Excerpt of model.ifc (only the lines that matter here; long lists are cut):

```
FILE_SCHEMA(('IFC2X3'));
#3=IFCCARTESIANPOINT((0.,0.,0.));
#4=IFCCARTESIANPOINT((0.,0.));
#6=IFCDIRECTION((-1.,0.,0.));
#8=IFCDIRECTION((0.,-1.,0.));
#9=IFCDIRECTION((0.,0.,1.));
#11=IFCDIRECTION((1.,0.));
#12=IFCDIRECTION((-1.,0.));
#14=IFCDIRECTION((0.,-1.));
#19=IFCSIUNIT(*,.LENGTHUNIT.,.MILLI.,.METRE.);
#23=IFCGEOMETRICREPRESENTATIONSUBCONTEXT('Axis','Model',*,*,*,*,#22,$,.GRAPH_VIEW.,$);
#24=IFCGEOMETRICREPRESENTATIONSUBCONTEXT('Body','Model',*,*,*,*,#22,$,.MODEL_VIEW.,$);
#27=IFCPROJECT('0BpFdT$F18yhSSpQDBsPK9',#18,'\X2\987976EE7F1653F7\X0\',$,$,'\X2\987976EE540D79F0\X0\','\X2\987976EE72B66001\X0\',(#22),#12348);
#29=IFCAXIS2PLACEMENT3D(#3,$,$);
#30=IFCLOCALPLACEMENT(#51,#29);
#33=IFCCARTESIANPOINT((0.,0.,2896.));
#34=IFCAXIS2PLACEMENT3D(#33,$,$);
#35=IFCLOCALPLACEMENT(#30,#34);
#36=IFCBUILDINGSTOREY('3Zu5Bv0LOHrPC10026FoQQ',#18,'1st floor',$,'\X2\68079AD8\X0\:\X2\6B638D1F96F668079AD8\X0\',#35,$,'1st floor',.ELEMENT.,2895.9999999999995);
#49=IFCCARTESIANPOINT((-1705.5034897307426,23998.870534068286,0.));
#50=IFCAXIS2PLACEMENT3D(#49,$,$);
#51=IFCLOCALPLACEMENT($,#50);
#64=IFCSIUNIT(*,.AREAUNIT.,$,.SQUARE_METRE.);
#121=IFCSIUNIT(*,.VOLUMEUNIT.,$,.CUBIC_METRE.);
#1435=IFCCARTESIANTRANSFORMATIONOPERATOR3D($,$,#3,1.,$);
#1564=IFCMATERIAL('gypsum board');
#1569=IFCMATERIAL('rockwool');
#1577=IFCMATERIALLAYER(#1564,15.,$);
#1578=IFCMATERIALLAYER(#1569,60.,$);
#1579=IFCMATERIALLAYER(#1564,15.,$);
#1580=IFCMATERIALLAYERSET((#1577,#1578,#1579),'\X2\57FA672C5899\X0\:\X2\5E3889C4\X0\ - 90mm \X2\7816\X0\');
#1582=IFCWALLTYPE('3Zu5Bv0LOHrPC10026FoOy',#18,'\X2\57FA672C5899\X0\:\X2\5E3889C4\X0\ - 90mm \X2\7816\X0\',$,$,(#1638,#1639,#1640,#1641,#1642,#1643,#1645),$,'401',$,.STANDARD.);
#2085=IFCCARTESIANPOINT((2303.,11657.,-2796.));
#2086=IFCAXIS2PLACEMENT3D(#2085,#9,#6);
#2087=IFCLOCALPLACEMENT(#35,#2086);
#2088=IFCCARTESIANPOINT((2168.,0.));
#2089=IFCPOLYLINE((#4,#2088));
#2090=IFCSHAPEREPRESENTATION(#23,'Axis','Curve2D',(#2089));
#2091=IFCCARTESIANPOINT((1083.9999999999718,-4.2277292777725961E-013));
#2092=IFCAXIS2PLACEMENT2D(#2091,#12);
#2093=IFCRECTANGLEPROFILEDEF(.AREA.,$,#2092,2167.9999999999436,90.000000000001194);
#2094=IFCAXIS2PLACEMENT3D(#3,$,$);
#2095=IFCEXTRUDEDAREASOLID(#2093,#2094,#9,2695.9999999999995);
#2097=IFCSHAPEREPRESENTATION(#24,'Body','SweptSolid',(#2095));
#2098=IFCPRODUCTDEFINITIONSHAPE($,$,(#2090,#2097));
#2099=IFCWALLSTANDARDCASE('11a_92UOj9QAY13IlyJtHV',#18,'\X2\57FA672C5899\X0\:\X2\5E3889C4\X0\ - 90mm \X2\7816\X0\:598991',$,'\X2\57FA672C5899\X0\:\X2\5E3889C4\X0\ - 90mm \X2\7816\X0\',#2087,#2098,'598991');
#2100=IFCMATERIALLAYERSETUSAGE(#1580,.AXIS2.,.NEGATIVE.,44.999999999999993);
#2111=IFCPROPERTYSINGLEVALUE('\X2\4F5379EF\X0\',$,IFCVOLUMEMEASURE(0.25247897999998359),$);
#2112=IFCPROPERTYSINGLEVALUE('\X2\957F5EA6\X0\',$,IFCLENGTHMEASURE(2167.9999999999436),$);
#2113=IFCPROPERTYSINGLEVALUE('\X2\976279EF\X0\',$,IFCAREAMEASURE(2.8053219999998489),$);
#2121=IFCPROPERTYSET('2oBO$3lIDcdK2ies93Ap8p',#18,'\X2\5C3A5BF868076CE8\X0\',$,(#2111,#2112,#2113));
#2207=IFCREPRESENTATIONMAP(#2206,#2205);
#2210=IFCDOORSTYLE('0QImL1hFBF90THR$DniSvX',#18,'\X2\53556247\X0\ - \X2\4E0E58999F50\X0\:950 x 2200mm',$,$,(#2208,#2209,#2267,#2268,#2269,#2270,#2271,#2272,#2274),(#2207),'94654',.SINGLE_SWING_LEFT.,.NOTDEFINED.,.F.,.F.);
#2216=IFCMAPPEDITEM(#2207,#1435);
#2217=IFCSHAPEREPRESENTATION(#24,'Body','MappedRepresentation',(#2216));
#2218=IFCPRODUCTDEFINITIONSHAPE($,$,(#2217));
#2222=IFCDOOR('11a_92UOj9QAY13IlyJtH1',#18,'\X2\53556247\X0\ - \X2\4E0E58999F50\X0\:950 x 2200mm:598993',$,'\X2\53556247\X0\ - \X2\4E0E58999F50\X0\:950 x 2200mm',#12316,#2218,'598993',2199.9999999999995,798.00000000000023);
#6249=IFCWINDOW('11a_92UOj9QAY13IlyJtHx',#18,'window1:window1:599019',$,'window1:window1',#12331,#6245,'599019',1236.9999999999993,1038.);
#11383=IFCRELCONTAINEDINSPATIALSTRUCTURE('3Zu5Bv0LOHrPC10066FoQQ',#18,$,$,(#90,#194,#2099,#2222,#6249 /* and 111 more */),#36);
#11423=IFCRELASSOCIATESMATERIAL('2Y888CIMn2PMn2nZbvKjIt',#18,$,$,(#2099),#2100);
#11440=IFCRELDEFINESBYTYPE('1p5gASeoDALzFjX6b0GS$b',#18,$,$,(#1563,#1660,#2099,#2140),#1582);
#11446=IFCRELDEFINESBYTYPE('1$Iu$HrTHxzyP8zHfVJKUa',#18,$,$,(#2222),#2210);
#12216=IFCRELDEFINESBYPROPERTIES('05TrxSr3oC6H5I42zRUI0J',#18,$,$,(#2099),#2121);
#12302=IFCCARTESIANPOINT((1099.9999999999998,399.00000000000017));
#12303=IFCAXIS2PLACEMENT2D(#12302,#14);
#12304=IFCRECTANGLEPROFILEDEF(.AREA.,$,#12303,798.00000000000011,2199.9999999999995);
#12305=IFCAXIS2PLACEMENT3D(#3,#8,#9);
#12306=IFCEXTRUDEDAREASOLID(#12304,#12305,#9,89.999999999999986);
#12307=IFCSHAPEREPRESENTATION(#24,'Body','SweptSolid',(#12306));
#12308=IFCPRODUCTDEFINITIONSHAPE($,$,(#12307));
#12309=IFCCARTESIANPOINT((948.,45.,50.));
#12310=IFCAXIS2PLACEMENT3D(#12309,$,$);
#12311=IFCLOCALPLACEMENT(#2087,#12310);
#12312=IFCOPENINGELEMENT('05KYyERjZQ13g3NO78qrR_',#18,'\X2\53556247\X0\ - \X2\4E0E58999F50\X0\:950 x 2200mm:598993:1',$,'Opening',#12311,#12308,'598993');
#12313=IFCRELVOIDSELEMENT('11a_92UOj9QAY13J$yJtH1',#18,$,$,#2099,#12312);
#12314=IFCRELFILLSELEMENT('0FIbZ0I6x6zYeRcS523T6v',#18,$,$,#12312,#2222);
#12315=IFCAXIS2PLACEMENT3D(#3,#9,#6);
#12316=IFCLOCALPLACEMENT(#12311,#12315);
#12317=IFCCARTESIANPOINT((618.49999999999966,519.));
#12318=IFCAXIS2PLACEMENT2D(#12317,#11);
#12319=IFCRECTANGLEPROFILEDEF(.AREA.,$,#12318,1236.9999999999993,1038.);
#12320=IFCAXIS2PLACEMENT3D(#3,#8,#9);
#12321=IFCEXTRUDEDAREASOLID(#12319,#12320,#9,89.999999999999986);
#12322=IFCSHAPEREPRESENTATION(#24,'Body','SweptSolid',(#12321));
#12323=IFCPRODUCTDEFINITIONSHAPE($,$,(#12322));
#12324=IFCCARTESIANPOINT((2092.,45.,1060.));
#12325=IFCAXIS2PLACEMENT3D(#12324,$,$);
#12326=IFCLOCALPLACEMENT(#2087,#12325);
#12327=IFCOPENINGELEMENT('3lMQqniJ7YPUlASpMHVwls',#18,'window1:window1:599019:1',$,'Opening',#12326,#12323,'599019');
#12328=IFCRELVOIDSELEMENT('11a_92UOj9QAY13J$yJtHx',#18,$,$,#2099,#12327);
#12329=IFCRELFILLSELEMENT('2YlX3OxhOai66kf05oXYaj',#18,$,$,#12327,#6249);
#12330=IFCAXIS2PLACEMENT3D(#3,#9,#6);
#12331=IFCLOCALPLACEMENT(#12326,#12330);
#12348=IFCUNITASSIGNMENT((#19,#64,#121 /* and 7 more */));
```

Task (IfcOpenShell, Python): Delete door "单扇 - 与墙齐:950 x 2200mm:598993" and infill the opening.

```python
import ifcopenshell
import ifcopenshell.api.feature
import ifcopenshell.api.pset
import ifcopenshell.api.root
import ifcopenshell.geom
import ifcopenshell.util.element
import ifcopenshell.util.shape
import ifcopenshell.util.unit

model = ifcopenshell.open("model.ifc")
area_scale = ifcopenshell.util.unit.calculate_unit_scale(model, "AREAUNIT")
volume_scale = ifcopenshell.util.unit.calculate_unit_scale(model, "VOLUMEUNIT")
settings = ifcopenshell.geom.settings()


def volume(element):
    """Net volume in cubic metres, openings subtracted."""
    shape = ifcopenshell.geom.create_shape(settings, element)
    return ifcopenshell.util.shape.get_volume(shape.geometry)


door = model.by_guid("11a_92UOj9QAY13IlyJtH1")
opening = door.FillsVoids[0].RelatingOpeningElement
wall = opening.VoidsElements[0].RelatingBuildingElement
before = volume(wall)

ifcopenshell.api.root.remove_product(model, product=door)
ifcopenshell.api.feature.remove_feature(model, feature=opening)

after = volume(wall)
thickness = 0.09  # wall thickness in metres

# Update the wall's stored quantities.
pset = model.by_id(ifcopenshell.util.element.get_pset(wall, "尺寸标注", should_inherit=False)["id"])
ifcopenshell.api.pset.edit_pset(model, pset=pset, properties={
    "体积": model.create_entity("IfcVolumeMeasure", after / volume_scale),
    "面积": model.create_entity("IfcAreaMeasure", after / thickness / area_scale),
})

print(f"wall volume {before:.3f} -> {after:.3f} m3")

model.write("model_edited.ifc")
```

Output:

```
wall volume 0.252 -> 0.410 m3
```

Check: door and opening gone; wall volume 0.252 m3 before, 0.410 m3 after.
